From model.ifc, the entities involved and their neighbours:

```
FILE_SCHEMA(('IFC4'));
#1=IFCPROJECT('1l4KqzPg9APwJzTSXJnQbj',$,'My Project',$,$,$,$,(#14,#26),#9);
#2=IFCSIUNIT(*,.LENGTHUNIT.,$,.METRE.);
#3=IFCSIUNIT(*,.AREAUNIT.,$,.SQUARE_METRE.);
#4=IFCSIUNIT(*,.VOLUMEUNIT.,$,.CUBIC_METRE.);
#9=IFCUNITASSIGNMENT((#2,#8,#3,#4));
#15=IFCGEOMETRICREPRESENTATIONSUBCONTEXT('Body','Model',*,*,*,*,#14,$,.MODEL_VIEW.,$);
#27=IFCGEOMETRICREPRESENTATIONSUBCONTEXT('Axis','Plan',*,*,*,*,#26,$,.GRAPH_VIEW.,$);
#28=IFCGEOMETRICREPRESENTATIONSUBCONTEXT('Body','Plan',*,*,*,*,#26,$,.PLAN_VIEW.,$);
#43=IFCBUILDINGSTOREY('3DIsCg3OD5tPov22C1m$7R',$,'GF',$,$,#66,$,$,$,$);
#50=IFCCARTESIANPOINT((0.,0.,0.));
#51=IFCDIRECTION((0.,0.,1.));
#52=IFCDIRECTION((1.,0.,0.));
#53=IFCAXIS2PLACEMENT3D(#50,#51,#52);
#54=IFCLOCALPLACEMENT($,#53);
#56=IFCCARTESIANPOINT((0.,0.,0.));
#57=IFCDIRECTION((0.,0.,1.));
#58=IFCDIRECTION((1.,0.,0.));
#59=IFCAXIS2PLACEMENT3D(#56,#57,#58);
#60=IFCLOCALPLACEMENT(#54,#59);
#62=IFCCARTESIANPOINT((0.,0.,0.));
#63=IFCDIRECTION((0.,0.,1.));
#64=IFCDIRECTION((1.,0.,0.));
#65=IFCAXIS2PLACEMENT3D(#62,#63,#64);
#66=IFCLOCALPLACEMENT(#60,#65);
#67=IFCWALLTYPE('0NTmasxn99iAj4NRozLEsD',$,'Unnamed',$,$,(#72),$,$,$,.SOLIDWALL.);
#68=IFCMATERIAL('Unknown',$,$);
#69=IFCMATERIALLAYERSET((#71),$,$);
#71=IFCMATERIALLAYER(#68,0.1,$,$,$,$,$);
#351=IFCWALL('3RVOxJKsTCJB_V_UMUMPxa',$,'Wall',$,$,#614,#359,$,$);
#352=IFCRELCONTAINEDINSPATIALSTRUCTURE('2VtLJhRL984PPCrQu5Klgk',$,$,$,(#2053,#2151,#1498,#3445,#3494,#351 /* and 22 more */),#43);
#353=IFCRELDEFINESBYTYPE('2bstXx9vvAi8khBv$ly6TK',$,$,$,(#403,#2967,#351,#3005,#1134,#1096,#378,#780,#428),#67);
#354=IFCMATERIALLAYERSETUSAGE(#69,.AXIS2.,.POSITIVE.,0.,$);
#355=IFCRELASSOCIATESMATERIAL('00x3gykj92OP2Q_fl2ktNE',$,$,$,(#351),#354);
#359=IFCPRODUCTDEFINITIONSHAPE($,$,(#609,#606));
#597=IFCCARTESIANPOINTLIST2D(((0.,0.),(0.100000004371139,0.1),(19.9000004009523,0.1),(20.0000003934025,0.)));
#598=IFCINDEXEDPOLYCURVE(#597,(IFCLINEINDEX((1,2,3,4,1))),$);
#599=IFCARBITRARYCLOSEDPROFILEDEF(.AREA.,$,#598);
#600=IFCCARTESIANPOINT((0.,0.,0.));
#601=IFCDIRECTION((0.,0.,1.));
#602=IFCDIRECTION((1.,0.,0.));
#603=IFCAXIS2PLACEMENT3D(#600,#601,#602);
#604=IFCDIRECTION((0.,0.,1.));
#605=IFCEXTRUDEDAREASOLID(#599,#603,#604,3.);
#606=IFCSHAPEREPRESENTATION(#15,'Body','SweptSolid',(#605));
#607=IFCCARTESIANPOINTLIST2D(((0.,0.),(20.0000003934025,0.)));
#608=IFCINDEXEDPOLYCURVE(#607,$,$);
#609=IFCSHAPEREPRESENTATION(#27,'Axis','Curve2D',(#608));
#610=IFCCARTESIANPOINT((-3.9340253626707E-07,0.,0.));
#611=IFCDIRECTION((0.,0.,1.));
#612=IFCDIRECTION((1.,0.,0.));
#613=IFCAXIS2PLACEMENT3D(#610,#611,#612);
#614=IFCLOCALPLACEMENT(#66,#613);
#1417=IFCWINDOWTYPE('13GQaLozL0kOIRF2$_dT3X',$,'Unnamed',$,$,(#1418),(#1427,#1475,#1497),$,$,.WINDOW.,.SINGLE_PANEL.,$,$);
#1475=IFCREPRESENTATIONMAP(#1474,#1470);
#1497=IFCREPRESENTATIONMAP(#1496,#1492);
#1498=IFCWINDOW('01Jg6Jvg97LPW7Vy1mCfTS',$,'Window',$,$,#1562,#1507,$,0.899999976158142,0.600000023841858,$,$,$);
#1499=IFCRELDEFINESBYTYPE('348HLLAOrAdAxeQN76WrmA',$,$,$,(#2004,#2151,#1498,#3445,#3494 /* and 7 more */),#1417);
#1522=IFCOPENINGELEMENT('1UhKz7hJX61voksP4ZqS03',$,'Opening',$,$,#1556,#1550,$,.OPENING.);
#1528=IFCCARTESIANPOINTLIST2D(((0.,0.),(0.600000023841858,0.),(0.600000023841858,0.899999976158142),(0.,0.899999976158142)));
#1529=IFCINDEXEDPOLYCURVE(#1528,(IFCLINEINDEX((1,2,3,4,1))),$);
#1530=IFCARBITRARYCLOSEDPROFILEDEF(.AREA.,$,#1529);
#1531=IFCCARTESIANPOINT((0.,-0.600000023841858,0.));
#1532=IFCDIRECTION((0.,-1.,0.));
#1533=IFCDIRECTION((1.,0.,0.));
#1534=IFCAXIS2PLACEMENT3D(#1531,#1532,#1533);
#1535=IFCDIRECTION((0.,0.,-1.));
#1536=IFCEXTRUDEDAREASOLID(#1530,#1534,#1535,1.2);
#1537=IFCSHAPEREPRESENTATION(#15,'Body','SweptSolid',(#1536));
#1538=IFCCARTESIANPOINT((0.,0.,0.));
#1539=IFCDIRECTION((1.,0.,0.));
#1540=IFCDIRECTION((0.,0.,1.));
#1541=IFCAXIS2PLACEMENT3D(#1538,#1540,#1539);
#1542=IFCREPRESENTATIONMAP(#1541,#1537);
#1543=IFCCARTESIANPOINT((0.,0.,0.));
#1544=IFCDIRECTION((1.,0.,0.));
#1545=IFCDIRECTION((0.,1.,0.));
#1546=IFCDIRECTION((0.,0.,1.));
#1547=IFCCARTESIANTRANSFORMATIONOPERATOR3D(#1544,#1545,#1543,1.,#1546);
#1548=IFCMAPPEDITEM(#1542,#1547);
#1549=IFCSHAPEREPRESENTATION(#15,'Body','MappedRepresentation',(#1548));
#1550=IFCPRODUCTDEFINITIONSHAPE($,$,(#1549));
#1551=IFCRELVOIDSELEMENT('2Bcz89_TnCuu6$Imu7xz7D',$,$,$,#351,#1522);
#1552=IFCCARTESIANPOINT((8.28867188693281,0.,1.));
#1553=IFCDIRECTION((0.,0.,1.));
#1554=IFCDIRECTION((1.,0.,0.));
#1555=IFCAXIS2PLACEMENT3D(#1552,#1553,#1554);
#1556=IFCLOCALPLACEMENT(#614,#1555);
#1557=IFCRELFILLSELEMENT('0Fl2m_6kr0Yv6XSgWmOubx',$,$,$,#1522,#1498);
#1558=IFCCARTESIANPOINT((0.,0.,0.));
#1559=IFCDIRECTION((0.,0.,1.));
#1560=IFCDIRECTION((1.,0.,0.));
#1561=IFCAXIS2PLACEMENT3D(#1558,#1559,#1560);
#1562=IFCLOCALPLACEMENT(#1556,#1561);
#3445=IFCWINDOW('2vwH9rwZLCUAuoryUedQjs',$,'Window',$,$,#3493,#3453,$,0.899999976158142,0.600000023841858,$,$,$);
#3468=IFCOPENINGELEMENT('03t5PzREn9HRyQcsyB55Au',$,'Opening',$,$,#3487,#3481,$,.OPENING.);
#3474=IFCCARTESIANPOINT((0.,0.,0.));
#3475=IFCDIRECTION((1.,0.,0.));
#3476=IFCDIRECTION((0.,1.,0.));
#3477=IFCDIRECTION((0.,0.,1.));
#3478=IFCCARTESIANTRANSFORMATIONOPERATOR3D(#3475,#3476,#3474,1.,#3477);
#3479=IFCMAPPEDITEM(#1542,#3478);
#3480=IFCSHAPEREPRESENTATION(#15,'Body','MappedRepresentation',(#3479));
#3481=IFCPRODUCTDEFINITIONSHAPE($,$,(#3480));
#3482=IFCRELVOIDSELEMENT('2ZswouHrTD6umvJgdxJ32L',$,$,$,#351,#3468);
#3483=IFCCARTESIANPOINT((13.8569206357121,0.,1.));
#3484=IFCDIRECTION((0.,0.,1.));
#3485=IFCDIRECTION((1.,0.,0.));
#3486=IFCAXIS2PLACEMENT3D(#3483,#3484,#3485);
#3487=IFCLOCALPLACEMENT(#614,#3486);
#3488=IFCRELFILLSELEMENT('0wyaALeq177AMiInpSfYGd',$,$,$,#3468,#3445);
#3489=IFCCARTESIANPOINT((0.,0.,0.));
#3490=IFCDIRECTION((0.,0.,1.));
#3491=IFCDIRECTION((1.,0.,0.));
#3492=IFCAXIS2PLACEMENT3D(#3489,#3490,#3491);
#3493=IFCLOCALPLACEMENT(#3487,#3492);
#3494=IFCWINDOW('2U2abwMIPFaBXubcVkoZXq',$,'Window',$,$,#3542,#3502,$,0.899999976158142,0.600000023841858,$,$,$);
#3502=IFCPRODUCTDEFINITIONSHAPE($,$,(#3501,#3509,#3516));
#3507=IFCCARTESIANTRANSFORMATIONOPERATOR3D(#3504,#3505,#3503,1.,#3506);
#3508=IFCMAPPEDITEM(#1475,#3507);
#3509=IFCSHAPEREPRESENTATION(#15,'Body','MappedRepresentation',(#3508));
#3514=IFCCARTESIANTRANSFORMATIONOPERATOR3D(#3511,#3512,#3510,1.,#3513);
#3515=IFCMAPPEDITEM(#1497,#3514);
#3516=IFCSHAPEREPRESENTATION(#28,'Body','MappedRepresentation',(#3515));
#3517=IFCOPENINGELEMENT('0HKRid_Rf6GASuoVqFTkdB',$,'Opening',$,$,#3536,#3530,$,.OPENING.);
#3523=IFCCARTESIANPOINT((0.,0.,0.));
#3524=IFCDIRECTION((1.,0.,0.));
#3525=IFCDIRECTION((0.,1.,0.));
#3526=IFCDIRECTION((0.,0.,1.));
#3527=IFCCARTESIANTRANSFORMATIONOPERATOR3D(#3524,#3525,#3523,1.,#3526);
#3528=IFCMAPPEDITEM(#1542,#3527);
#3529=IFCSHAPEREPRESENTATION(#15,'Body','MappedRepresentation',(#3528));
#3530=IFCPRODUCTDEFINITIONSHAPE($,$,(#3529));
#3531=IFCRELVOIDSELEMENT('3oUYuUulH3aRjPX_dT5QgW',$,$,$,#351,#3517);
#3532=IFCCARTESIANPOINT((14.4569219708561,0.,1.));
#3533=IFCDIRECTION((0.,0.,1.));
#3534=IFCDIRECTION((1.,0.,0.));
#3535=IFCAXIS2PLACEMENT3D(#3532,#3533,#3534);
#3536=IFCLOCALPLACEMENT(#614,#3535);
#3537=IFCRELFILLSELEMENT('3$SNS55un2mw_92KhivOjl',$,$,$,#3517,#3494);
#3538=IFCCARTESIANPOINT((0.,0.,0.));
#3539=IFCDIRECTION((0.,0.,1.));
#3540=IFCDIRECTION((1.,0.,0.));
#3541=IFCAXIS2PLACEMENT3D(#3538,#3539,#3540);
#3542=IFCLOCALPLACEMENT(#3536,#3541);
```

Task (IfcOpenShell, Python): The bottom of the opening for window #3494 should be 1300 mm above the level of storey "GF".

```python
import numpy as np
import ifcopenshell
import ifcopenshell.api.geometry
import ifcopenshell.geom
import ifcopenshell.util.element
import ifcopenshell.util.placement
import ifcopenshell.util.shape
import ifcopenshell.util.unit

model = ifcopenshell.open("model.ifc")
unit_scale = ifcopenshell.util.unit.calculate_unit_scale(model)

window = model.by_guid("2U2abwMIPFaBXubcVkoZXq")
opening = window.FillsVoids[0].RelatingOpeningElement
storey = ifcopenshell.util.element.get_container(window, ifc_class="IfcBuildingStorey")
level = ifcopenshell.util.placement.get_local_placement(storey.ObjectPlacement)[2, 3]

# The opening's origin need not be at the sill, so measure its lowest point.
shape = ifcopenshell.geom.create_shape(ifcopenshell.geom.settings(), opening)
bottom = ifcopenshell.util.shape.get_shape_bottom_elevation(shape, shape.geometry) / unit_scale
dz = level + 1.3 / unit_scale - bottom

shift = np.array([0.0, 0.0, dz])
# The window is placed relative to its opening, so it follows when the opening moves.
matrix = ifcopenshell.util.placement.get_local_placement(opening.ObjectPlacement)
matrix[:3, 3] += shift
ifcopenshell.api.geometry.edit_object_placement(
    model, product=opening, matrix=matrix, is_si=False, should_transform_children=True
)

print(f"moved by {dz * unit_scale:+.3f} m")

model.write("model_updated.ifc")
```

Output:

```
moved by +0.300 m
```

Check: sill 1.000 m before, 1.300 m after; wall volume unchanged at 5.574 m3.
